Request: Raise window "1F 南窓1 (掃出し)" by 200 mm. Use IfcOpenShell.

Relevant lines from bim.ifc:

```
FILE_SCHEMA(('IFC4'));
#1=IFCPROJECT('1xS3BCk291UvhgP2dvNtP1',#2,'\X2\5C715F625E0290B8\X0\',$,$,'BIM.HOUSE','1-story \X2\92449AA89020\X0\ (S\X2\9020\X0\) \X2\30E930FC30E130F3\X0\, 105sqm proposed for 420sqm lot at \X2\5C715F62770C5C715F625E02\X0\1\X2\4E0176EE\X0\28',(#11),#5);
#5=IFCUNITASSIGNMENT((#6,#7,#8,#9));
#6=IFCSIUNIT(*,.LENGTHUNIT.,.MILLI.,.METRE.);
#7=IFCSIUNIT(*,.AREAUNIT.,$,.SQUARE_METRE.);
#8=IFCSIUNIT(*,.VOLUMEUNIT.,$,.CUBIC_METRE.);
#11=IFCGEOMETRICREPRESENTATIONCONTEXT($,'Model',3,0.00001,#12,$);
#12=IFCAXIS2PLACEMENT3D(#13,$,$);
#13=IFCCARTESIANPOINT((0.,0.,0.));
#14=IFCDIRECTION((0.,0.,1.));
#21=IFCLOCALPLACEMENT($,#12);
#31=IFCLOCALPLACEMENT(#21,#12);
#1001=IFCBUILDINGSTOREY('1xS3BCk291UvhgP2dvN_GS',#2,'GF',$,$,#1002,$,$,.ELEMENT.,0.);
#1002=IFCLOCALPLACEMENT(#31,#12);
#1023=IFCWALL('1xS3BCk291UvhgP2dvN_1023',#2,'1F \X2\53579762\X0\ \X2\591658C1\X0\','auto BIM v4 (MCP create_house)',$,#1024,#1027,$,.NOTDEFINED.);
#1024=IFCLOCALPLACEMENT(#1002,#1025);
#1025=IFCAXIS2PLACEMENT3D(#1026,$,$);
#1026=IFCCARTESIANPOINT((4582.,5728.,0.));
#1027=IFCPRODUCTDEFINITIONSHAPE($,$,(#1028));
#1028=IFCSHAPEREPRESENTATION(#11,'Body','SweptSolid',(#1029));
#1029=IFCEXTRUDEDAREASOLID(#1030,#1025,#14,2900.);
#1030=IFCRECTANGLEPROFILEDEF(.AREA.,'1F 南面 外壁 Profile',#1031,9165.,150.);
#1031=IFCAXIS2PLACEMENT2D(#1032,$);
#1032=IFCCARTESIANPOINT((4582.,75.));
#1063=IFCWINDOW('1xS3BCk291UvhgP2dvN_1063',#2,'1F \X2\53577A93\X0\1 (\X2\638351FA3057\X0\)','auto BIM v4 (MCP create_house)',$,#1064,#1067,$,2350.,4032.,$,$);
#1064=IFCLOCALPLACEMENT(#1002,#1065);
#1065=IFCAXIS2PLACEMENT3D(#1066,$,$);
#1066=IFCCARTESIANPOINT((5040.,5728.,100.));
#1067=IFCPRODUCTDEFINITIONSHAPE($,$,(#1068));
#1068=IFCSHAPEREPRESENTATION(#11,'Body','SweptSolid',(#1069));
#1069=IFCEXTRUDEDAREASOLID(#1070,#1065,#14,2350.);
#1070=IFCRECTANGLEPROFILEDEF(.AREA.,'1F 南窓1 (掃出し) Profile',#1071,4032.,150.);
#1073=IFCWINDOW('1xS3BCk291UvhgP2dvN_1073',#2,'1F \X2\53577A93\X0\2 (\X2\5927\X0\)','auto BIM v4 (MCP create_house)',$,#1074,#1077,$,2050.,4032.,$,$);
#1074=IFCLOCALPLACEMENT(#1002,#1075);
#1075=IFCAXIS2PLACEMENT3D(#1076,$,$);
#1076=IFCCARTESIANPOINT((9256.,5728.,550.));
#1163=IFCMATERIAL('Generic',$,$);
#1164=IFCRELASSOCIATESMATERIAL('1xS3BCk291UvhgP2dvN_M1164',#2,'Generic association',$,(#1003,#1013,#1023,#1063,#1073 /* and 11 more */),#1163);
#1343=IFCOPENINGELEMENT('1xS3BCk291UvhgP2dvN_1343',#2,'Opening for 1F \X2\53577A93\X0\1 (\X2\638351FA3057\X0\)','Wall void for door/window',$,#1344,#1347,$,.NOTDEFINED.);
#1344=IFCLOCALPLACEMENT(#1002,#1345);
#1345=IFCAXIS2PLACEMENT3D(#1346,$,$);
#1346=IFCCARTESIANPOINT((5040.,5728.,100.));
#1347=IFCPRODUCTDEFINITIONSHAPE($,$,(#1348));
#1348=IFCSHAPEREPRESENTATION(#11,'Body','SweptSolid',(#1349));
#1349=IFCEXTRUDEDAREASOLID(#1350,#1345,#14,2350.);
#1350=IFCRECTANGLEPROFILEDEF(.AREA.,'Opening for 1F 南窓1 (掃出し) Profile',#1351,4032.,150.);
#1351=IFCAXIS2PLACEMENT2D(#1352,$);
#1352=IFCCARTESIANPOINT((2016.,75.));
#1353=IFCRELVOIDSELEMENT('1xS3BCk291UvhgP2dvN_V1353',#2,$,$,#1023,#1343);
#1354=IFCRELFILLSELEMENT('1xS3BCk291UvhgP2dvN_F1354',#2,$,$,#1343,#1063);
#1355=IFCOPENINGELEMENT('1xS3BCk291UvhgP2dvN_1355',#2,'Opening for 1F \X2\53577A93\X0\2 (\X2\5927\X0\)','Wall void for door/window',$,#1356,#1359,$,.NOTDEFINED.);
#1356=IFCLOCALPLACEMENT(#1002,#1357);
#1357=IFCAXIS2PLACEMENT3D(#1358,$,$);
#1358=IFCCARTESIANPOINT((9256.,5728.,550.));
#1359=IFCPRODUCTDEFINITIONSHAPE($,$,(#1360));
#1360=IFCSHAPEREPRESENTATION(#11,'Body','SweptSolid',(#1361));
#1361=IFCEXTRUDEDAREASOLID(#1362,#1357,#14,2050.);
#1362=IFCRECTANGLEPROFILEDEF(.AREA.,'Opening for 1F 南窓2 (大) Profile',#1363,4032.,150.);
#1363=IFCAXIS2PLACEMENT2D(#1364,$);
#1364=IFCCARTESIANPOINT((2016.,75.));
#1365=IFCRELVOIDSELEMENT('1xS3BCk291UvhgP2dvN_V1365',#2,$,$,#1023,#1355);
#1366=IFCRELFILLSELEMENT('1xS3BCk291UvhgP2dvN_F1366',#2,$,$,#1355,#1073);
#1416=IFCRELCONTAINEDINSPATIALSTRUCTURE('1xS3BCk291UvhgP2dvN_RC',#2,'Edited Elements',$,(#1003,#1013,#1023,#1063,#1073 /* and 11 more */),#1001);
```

```python
import numpy as np
import ifcopenshell
import ifcopenshell.api.geometry
import ifcopenshell.util.placement
import ifcopenshell.util.unit

model = ifcopenshell.open("bim.ifc")
unit_scale = ifcopenshell.util.unit.calculate_unit_scale(model)

window = model.by_guid("1xS3BCk291UvhgP2dvN_1063")
opening = window.FillsVoids[0].RelatingOpeningElement
dz = 0.2 / unit_scale

shift = np.array([0.0, 0.0, dz])
# The window is not placed relative to its opening, so move both.
for product in (opening, window):
    matrix = ifcopenshell.util.placement.get_local_placement(product.ObjectPlacement)
    matrix[:3, 3] += shift
    ifcopenshell.api.geometry.edit_object_placement(model, product=product, matrix=matrix, is_si=False)

print(f"moved by {dz * unit_scale:+.3f} m")

model.write("bim-out.ifc")
```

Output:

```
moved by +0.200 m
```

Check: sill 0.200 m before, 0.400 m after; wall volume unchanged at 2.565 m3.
